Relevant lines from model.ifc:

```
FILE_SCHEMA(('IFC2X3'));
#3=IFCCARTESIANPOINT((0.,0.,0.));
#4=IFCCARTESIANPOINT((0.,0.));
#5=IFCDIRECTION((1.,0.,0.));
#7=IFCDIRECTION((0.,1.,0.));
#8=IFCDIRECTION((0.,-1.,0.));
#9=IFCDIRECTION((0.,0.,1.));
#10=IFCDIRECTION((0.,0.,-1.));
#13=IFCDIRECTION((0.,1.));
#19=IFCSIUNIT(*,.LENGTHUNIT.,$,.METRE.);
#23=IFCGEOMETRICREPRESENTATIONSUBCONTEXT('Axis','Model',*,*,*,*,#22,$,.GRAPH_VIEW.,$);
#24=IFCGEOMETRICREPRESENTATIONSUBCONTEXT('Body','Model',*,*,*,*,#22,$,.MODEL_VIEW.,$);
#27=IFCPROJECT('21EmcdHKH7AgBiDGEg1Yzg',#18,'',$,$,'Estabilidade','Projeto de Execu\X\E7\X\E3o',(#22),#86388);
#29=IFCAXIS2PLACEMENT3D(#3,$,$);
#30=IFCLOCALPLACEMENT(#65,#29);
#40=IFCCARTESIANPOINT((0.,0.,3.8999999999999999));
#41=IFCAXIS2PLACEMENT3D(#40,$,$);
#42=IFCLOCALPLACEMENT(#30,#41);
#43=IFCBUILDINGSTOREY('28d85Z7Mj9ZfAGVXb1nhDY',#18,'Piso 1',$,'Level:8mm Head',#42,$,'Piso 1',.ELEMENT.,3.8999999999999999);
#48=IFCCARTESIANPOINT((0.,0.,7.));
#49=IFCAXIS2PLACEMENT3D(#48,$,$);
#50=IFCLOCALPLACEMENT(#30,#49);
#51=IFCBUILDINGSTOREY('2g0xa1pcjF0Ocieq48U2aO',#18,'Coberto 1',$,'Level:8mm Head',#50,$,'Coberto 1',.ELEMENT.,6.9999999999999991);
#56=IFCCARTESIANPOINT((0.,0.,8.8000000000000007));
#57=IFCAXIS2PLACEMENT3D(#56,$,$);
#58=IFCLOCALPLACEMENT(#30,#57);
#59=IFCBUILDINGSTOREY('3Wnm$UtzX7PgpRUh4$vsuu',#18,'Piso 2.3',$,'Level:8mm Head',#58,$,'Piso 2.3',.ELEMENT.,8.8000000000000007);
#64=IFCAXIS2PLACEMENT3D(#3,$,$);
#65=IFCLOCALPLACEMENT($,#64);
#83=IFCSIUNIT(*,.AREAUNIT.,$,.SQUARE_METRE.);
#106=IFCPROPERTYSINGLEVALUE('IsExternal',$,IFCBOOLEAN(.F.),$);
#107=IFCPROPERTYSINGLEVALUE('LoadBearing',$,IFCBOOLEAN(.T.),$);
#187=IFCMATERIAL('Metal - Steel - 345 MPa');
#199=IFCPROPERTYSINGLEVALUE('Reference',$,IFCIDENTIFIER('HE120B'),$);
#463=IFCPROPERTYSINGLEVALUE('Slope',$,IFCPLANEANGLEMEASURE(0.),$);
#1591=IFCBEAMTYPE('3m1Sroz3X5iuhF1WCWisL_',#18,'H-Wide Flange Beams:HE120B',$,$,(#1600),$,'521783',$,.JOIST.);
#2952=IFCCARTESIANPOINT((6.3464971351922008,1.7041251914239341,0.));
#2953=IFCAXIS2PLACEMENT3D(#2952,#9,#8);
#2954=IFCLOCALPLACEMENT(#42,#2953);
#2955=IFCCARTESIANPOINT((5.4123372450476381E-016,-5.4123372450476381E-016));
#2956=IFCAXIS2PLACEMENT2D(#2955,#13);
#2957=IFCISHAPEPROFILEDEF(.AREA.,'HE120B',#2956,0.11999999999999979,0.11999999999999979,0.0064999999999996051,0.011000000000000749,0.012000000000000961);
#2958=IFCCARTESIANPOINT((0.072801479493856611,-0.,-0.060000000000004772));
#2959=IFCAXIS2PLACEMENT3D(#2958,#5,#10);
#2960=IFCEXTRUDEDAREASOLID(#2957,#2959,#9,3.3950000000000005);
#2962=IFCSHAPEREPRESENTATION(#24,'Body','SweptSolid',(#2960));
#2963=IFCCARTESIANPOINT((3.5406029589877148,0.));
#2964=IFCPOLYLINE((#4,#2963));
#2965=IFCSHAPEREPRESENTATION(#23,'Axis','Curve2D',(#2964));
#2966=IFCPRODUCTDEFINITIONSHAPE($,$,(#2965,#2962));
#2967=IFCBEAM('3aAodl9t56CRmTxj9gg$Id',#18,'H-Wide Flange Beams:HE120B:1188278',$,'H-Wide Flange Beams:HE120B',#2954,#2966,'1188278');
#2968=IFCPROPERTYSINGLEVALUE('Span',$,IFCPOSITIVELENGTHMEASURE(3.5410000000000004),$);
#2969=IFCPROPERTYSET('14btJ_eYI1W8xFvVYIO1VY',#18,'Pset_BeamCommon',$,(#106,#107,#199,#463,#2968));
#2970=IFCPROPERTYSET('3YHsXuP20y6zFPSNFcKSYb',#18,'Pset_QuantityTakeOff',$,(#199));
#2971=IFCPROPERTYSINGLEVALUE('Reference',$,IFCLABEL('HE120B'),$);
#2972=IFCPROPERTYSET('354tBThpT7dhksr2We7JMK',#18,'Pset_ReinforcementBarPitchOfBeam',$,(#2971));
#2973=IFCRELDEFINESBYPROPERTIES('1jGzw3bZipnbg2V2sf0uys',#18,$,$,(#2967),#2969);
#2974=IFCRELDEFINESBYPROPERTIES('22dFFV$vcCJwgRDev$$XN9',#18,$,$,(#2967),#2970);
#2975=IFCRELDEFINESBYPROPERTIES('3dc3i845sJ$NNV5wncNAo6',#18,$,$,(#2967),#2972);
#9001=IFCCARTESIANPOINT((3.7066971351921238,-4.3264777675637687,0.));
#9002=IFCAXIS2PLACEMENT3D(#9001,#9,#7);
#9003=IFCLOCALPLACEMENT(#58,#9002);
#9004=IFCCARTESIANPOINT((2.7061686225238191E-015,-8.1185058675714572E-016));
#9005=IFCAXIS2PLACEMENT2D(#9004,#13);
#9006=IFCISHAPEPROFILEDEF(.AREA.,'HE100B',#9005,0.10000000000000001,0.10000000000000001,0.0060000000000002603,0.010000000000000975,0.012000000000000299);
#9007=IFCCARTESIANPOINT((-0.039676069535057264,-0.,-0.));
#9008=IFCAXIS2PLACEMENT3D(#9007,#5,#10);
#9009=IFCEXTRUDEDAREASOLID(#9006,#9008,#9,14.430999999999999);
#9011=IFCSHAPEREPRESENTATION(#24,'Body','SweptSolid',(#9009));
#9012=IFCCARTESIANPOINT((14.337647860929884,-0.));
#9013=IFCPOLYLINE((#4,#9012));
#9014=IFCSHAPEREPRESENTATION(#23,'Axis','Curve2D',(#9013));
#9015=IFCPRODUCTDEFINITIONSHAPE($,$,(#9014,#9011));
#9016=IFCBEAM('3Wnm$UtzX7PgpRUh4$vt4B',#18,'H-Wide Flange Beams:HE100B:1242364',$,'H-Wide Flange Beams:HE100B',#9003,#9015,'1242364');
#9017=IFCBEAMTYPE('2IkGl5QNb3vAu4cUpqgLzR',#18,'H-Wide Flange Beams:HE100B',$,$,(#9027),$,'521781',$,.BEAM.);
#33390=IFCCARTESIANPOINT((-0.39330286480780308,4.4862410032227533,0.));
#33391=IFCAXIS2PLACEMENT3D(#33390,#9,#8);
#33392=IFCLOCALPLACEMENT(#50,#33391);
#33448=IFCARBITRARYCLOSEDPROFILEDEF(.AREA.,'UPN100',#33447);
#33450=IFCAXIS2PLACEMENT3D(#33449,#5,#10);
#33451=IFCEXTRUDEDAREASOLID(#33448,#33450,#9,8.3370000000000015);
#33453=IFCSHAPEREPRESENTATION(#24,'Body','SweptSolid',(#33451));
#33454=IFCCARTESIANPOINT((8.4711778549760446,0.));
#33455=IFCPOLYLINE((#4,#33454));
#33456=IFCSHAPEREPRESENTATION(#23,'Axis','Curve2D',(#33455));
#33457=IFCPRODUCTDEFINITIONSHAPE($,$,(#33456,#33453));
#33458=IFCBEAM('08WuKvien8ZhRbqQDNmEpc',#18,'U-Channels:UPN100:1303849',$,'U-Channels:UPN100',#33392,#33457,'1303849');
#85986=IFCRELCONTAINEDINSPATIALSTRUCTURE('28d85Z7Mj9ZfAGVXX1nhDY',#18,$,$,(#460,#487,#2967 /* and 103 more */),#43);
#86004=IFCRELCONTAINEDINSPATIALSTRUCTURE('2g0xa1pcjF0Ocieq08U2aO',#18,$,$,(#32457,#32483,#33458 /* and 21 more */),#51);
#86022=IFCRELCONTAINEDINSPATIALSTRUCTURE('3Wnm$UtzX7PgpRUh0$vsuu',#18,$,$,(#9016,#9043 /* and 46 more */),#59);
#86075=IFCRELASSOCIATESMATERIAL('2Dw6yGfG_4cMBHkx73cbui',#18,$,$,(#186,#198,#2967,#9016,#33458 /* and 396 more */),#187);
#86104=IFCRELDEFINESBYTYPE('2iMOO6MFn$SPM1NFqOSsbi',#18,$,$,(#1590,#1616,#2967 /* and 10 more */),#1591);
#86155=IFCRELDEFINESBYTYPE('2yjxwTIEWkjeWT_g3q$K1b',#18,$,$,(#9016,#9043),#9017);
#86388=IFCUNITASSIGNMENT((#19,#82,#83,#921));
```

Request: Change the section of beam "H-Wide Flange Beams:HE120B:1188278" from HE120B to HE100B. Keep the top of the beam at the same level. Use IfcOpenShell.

```python
import ifcopenshell
import ifcopenshell.api.pset
import ifcopenshell.api.type
import ifcopenshell.util.element
import ifcopenshell.util.representation

model = ifcopenshell.open("model.ifc")

member = model.by_guid("3aAodl9t56CRmTxj9gg$Id")
source = next(p for p in model.by_type("IfcIShapeProfileDef") if p.ProfileName == "HE100B")

body = ifcopenshell.util.representation.get_representation(member, "Model", "Body")
solid = body.Items[0]
old_profile = solid.SweptArea

# Copy the section's sizes but keep this member's own profile position.
profile = ifcopenshell.util.element.copy(model, source)
# Profiles are centred, so shift by half the change in depth to hold the top.
shift = (old_profile.OverallDepth - profile.OverallDepth) / 2
x, y = old_profile.Position.Location.Coordinates
up = (-1.0, 0.0)  # upwards, in the solid's own plane
location = model.createIfcCartesianPoint((x + up[0] * shift, y + up[1] * shift))
profile.Position = model.createIfcAxis2Placement2D(location, old_profile.Position.RefDirection)
solid.SweptArea = profile
if not model.get_total_inverses(old_profile):
    ifcopenshell.util.element.remove_deep2(model, old_profile)

new_type = model.by_guid("2IkGl5QNb3vAu4cUpqgLzR")
ifcopenshell.api.type.assign_type(
    model, related_objects=[member], relating_type=new_type, should_map_representations=False
)
member.Name = member.Name.replace("HE120B", "HE100B")
member.ObjectType = "H-Wide Flange Beams:HE100B"
pset = model.by_id(ifcopenshell.util.element.get_pset(member, "Pset_BeamCommon", should_inherit=False)["id"])
ifcopenshell.api.pset.edit_pset(model, pset=pset, properties={"Reference": "HE100B"})
pset = model.by_id(ifcopenshell.util.element.get_pset(member, "Pset_QuantityTakeOff", should_inherit=False)["id"])
ifcopenshell.api.pset.edit_pset(model, pset=pset, properties={"Reference": "HE100B"})
pset = model.by_id(ifcopenshell.util.element.get_pset(member, "Pset_ReinforcementBarPitchOfBeam", should_inherit=False)["id"])
ifcopenshell.api.pset.edit_pset(model, pset=pset, properties={"Reference": "HE100B"})

print(solid.SweptArea)

model.write("model-out.ifc")
```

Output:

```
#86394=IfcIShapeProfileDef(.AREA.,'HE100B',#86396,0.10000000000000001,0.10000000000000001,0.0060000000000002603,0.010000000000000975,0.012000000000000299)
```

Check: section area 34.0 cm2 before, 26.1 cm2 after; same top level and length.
